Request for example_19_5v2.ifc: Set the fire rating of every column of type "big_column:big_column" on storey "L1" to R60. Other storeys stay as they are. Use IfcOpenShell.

First a look at what the model holds.

```python
import ifcopenshell
import ifcopenshell.util.element

model = ifcopenshell.open("example_19_5v2.ifc")
print(model.schema)
storey = next(s for s in model.by_type("IfcBuildingStorey") if s.Name == "L1")
columns = [e for e in ifcopenshell.util.element.get_decomposition(storey) if e.is_a("IfcColumn")]
seen = {}
for e in columns:
    element_type = ifcopenshell.util.element.get_type(e)
    key = (element_type.Name if element_type != e and element_type else None, ifcopenshell.util.element.get_pset(e, "Pset_ColumnCommon", "FireRating"))
    seen[key] = seen.get(key, 0) + 1
for (name, value), count in sorted(seen.items(), key=str):
    print(count, "x", name, "|", value)
```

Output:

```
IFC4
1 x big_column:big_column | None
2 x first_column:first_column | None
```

```python
import ifcopenshell
import ifcopenshell.api.pset
import ifcopenshell.util.element

model = ifcopenshell.open("example_19_5v2.ifc")

storey = next(s for s in model.by_type("IfcBuildingStorey") if s.Name == "L1")
columns = [e for e in ifcopenshell.util.element.get_decomposition(storey) if e.is_a("IfcColumn")]

count = 0
for e in columns:
    element_type = ifcopenshell.util.element.get_type(e)
    if element_type in (None, e) or element_type.Name != "big_column:big_column":
        continue
    # add_pset returns the element's existing set when there is one.
    pset = ifcopenshell.api.pset.add_pset(model, product=e, name="Pset_ColumnCommon")
    ifcopenshell.api.pset.edit_pset(model, pset=pset, properties={"FireRating": "R60"})
    count += 1

print(count, "columns updated")

model.write("example_19_5v2_rev.ifc")
```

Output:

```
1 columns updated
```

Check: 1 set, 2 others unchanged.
